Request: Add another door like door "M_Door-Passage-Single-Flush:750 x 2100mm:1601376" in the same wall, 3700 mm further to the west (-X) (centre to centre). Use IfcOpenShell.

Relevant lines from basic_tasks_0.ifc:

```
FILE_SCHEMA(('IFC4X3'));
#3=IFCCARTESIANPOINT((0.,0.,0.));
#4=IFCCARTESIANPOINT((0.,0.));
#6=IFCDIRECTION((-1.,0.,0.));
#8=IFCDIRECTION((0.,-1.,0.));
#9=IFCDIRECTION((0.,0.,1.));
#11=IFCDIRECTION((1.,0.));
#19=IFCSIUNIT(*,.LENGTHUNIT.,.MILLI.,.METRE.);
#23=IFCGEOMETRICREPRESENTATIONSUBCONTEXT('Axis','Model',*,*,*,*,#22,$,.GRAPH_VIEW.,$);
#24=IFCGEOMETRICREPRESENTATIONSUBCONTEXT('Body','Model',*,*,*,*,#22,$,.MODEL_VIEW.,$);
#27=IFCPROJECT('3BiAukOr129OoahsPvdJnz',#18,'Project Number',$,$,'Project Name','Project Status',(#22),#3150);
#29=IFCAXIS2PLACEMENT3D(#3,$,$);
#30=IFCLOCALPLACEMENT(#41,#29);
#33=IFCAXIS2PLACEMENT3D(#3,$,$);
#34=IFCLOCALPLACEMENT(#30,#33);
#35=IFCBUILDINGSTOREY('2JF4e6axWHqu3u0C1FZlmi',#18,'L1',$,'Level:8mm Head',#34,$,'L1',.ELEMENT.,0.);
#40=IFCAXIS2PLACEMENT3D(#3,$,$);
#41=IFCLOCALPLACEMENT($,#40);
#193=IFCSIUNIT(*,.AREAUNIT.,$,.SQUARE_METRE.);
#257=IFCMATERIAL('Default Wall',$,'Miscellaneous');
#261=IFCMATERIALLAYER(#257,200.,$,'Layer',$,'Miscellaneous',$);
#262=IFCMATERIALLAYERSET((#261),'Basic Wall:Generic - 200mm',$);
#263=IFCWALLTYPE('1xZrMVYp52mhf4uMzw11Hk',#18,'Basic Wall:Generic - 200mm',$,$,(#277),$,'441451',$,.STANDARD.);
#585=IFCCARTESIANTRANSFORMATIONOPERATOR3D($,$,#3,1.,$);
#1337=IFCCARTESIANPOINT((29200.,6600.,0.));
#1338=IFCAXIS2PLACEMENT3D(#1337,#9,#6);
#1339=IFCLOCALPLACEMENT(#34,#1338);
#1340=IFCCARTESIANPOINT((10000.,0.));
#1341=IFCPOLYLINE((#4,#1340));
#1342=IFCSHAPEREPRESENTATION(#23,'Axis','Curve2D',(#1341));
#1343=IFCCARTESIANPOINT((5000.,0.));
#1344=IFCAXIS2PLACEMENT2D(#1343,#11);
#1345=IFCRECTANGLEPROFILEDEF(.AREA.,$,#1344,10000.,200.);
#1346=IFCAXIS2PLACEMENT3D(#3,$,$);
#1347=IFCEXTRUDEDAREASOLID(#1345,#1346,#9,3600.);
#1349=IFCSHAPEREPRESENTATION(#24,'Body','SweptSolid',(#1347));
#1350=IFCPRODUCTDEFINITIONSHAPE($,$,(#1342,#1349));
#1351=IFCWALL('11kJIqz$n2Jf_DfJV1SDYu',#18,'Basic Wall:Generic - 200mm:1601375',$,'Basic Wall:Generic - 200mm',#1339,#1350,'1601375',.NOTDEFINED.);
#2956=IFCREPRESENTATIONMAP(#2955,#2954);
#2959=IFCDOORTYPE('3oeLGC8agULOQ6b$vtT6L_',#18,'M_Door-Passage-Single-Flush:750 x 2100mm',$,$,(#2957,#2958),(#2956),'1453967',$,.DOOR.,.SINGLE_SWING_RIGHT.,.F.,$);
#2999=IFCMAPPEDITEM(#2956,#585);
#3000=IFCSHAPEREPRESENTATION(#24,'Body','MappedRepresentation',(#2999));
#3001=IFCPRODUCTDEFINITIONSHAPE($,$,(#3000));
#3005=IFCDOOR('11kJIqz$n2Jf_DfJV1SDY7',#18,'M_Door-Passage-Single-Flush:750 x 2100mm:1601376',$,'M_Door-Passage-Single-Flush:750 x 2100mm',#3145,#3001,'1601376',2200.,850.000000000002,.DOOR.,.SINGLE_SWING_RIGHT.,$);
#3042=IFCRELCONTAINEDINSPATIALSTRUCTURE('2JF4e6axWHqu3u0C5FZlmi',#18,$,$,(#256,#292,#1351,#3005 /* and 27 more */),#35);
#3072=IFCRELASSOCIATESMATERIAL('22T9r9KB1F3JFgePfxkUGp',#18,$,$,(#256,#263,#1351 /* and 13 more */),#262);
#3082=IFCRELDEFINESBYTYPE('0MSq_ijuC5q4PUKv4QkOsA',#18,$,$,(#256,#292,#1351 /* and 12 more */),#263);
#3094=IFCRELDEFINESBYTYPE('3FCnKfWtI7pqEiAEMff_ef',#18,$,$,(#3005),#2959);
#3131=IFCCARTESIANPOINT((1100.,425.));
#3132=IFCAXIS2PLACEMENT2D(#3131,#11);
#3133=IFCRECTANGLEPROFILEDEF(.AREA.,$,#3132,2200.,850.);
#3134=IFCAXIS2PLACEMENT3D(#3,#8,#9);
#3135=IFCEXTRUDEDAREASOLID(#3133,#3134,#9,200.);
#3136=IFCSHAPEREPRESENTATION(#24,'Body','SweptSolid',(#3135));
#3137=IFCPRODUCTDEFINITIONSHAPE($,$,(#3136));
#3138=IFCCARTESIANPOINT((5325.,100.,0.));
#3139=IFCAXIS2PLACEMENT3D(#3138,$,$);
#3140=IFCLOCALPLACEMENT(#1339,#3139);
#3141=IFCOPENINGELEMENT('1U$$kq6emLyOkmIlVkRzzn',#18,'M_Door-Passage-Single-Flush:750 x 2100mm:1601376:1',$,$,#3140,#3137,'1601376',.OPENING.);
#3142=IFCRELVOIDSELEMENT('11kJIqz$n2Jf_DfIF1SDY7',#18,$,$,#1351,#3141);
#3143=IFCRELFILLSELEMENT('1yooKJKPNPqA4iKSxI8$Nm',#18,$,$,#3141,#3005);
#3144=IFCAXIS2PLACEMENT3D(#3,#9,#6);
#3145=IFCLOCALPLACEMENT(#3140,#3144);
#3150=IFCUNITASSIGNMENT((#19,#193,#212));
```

```python
import ifcopenshell
import ifcopenshell.api.feature
import ifcopenshell.api.geometry
import ifcopenshell.api.root
import ifcopenshell.geom
import ifcopenshell.util.element
import ifcopenshell.util.placement
import ifcopenshell.util.shape
import ifcopenshell.util.unit

model = ifcopenshell.open("basic_tasks_0.ifc")
unit_scale = ifcopenshell.util.unit.calculate_unit_scale(model)
settings = ifcopenshell.geom.settings()


def volume(element):
    """Net volume in cubic metres, openings subtracted."""
    shape = ifcopenshell.geom.create_shape(settings, element)
    return ifcopenshell.util.shape.get_volume(shape.geometry)


def reuse_history(source, copy):
    """copy_class also copies each property set's owner history, people and application; keep the originals."""
    for rel in copy.IsDefinedBy:
        if rel.is_a("IfcRelDefinesByProperties") and (history := rel.RelatingPropertyDefinition.OwnerHistory):
            rel.RelatingPropertyDefinition.OwnerHistory = source.OwnerHistory
            ifcopenshell.util.element.remove_deep2(model, history)


door = model.by_guid("11kJIqz$n2Jf_DfJV1SDY7")
opening = door.FillsVoids[0].RelatingOpeningElement
wall = opening.VoidsElements[0].RelatingBuildingElement
before = volume(wall)
shift = ifcopenshell.util.placement.get_local_placement(wall.ObjectPlacement)[:3, 0] * 3.7 / unit_scale

# copy_class copies the void relationship, type, container and properties, but no geometry.
new_opening = ifcopenshell.api.root.copy_class(model, product=opening)
new_opening.Representation = ifcopenshell.util.element.copy_deep(
    model, opening.Representation, exclude=["IfcGeometricRepresentationContext", "IfcRepresentationMap"]
)
new_opening.Name = "M_Door-Passage-Single-Flush:750 x 2100mm"
new_opening.Tag = None
new_door = ifcopenshell.api.root.copy_class(model, product=door)
new_door.Representation = ifcopenshell.util.element.copy_deep(
    model, door.Representation, exclude=["IfcGeometricRepresentationContext", "IfcRepresentationMap"]
)
new_door.Name = "M_Door-Passage-Single-Flush:750 x 2100mm"
new_door.Tag = None
reuse_history(door, new_door)
ifcopenshell.api.feature.add_filling(model, opening=new_opening, element=new_door)

for old, new in ((opening, new_opening), (door, new_door)):
    matrix = ifcopenshell.util.placement.get_local_placement(old.ObjectPlacement)
    matrix[:3, 3] += shift
    ifcopenshell.api.geometry.edit_object_placement(model, product=new, matrix=matrix, is_si=False)

after = volume(wall)

print(f"wall volume {before:.3f} -> {after:.3f} m3")

model.write("basic_tasks_0_v2.ifc")
```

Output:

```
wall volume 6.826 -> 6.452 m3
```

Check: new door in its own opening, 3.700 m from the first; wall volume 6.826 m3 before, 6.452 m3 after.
